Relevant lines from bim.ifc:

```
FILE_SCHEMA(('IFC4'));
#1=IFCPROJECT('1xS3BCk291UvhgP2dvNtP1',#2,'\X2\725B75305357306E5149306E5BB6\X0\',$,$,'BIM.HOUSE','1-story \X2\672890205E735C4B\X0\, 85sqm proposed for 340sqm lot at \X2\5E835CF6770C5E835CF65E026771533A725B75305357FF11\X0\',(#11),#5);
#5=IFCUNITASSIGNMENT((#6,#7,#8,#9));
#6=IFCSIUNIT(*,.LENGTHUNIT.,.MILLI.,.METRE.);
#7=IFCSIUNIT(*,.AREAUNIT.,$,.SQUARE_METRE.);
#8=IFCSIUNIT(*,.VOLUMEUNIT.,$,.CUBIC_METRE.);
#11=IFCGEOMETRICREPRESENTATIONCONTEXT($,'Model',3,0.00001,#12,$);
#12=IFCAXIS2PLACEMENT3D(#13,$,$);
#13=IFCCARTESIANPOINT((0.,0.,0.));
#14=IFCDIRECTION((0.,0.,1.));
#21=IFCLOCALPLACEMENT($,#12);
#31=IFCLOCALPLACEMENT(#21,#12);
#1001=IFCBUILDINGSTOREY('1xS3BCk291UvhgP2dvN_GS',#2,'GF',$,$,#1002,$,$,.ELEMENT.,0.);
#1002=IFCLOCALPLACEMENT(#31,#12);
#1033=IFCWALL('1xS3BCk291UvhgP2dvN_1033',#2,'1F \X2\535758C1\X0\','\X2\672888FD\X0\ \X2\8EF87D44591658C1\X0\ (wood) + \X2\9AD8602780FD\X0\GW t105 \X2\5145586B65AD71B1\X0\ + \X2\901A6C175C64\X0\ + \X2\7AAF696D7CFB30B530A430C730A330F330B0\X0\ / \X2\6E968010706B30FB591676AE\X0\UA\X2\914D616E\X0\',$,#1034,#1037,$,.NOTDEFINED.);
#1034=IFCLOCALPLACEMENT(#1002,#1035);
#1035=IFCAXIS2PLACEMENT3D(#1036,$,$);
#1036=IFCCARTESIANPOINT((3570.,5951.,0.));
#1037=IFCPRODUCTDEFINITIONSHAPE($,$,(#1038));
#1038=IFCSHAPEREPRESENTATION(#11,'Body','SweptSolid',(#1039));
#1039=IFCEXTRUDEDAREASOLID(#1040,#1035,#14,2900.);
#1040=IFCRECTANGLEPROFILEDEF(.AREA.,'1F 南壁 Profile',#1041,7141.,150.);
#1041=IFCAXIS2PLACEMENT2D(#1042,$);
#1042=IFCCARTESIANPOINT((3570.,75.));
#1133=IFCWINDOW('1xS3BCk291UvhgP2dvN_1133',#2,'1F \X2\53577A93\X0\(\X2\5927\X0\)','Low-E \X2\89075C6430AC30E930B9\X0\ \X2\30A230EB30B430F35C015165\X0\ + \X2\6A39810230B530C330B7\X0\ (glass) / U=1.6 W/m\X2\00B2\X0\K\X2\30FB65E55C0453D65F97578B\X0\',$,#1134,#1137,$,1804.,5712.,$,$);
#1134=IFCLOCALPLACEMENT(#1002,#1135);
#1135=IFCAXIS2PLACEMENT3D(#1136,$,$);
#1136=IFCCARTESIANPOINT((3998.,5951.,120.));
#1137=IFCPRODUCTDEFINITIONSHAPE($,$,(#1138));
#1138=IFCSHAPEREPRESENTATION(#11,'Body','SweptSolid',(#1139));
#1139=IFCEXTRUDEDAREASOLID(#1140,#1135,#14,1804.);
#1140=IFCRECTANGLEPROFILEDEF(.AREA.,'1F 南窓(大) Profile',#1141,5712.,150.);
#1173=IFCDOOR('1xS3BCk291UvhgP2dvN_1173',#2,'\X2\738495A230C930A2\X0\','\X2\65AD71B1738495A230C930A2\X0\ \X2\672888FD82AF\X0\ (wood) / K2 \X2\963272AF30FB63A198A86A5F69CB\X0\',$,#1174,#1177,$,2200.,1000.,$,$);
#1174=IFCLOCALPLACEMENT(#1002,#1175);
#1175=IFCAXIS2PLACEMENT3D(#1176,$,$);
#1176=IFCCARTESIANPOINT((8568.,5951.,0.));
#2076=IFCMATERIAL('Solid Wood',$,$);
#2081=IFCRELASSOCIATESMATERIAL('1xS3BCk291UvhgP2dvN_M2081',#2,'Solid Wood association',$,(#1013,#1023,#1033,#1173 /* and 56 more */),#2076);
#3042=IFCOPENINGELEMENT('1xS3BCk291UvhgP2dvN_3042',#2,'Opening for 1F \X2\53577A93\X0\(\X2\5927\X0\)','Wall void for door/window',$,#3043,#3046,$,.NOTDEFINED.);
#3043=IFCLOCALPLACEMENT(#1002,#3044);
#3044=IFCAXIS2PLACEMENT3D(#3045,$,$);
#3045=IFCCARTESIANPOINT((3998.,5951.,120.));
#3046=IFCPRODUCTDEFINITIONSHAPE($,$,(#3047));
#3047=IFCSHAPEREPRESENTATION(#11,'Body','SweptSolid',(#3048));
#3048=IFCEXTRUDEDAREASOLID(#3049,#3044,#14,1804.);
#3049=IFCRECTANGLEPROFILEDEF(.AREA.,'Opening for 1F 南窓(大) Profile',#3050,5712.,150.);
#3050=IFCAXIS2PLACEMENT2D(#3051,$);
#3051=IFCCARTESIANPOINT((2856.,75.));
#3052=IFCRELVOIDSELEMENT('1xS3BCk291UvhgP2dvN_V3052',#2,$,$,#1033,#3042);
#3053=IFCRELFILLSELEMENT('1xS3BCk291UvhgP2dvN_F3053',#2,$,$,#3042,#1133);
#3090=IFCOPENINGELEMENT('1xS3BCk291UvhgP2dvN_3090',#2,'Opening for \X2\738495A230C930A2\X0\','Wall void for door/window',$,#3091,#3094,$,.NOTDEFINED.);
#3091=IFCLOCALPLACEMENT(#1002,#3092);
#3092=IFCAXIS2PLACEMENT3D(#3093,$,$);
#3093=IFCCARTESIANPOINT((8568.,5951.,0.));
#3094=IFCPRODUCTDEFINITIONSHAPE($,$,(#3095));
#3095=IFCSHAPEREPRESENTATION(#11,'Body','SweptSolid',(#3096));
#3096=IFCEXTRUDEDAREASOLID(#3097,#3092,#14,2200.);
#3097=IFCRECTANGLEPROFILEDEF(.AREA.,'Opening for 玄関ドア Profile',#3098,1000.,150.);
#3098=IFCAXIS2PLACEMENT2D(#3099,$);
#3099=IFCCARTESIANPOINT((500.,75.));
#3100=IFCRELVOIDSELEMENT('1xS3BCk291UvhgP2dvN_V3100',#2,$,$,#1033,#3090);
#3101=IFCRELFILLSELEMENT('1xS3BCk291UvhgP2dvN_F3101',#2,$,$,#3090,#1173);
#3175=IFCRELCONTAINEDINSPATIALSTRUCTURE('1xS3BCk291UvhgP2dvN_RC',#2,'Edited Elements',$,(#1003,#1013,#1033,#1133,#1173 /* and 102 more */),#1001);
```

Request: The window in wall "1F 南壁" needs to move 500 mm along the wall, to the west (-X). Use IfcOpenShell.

```python
import ifcopenshell
import ifcopenshell.api.geometry
import ifcopenshell.util.placement
import ifcopenshell.util.unit

model = ifcopenshell.open("bim.ifc")
unit_scale = ifcopenshell.util.unit.calculate_unit_scale(model)

window = model.by_id(1133)
opening = window.FillsVoids[0].RelatingOpeningElement
wall = opening.VoidsElements[0].RelatingBuildingElement

wall_matrix = ifcopenshell.util.placement.get_local_placement(wall.ObjectPlacement)
shift = wall_matrix[:3, 0] * -0.5 / unit_scale
before = ifcopenshell.util.placement.get_local_placement(window.ObjectPlacement)[:3, 3].copy()

# The window is not placed relative to its opening, so move both.
for product in (opening, window):
    matrix = ifcopenshell.util.placement.get_local_placement(product.ObjectPlacement)
    matrix[:3, 3] += shift
    ifcopenshell.api.geometry.edit_object_placement(model, product=product, matrix=matrix, is_si=False)

after = ifcopenshell.util.placement.get_local_placement(window.ObjectPlacement)[:3, 3]
print("window moved by", (after - before).round(3) + 0.0)

model.write("bim_edited.ifc")
```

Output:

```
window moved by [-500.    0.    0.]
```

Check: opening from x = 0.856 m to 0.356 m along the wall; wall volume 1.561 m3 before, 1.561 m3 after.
